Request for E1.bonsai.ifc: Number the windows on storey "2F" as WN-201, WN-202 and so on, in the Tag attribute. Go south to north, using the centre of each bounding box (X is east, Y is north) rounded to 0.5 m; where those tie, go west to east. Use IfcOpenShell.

First a look at what the model holds.

```python
import ifcopenshell
import ifcopenshell.util.element
import ifcopenshell.util.placement

model = ifcopenshell.open("E1.bonsai.ifc")
print(model.schema)
storey = next(s for s in model.by_type("IfcBuildingStorey") if s.Name == "2F")
windows = [e for e in ifcopenshell.util.element.get_decomposition(storey) if e.is_a("IfcWindow")]
for e in sorted(windows, key=lambda e: e.id()):
    origin = ifcopenshell.util.placement.get_local_placement(e.ObjectPlacement)[:3, 3]
    print(e.id(), e.Tag, e.Name, origin.round(2) + 0.0, sep=" | ")
```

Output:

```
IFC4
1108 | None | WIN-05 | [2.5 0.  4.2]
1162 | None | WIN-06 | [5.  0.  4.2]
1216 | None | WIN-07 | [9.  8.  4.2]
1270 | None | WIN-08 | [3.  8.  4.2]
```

```python
import ifcopenshell
import ifcopenshell.geom
import ifcopenshell.util.element
import ifcopenshell.util.shape

model = ifcopenshell.open("E1.bonsai.ifc")
settings = ifcopenshell.geom.settings()
settings.set("use-world-coords", True)


def centre(element):
    shape = ifcopenshell.geom.create_shape(settings, element)
    return ifcopenshell.util.shape.get_bbox_centroid(shape.geometry)


storey = next(s for s in model.by_type("IfcBuildingStorey") if s.Name == "2F")
windows = [e for e in ifcopenshell.util.element.get_decomposition(storey) if e.is_a("IfcWindow")]

# Insertion points can sit at a corner or the storey origin, so sort by the geometry (in metres).
centres = {e: centre(e) for e in windows}
windows.sort(key=lambda e: (round(centres[e][1] / 0.5), centres[e][0]))

for i, e in enumerate(windows, start=1):
    number = f"WN-2{i:02d}"
    e.Tag = number
    print(e.id(), number)

model.write("E1.bonsai_v2.ifc")
```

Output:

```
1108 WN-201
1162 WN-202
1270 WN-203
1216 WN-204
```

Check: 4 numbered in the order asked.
